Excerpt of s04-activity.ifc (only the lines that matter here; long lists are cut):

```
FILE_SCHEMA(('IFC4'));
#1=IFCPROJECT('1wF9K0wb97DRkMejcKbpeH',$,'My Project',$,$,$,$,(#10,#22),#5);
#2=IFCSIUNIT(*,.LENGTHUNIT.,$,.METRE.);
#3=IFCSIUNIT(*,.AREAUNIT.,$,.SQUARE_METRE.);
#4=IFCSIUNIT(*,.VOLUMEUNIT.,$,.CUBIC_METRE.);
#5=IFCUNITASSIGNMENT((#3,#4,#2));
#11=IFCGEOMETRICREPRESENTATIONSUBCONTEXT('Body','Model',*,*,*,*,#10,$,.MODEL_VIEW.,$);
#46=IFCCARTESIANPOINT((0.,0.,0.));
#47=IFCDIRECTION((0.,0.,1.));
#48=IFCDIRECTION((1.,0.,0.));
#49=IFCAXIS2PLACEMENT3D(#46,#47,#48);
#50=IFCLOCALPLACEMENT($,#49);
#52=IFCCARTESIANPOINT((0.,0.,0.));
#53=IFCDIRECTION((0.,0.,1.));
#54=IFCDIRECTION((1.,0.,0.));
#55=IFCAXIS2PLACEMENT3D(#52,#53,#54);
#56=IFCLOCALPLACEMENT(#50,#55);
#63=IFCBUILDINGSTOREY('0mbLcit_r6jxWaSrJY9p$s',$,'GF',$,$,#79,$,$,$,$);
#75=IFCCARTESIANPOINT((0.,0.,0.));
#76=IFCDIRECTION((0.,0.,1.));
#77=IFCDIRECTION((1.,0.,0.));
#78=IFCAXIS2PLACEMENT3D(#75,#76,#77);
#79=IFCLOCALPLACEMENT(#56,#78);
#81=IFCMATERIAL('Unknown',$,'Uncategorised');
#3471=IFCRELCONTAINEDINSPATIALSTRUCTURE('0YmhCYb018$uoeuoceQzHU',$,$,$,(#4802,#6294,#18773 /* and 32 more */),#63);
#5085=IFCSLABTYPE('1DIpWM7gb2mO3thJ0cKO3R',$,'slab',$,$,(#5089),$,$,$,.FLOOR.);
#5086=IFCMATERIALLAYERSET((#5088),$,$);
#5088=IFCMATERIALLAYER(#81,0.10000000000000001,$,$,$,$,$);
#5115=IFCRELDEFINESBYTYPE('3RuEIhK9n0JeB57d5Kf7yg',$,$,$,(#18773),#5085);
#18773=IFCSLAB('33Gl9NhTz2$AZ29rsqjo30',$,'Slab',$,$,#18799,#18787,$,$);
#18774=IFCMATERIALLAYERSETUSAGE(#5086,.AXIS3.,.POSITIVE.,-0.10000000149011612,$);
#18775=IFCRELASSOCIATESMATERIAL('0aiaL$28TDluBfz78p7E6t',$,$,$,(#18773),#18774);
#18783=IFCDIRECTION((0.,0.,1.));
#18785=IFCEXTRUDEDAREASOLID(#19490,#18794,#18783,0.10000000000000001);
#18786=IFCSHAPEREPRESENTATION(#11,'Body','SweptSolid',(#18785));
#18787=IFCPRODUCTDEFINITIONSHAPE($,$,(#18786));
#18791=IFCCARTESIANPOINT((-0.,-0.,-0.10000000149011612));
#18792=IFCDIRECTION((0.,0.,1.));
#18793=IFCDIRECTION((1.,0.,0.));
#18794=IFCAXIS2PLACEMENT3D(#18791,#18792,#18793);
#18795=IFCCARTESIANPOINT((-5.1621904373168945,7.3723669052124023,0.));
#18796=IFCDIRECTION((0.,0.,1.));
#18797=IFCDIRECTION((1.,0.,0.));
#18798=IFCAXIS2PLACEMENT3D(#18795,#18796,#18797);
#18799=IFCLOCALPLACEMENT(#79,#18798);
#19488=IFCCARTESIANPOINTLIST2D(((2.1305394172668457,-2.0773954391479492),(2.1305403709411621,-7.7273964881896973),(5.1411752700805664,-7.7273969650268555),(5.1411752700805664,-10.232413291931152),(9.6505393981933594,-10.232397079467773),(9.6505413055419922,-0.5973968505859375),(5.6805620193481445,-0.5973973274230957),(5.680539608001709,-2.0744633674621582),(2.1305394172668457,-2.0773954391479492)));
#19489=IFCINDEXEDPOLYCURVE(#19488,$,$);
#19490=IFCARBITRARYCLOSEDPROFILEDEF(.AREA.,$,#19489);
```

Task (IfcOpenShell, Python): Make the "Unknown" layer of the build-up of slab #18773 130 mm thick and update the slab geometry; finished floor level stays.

```python
import ifcopenshell
import ifcopenshell.util.element
import ifcopenshell.util.representation
import ifcopenshell.util.unit

model = ifcopenshell.open("s04-activity.ifc")
unit_scale = ifcopenshell.util.unit.calculate_unit_scale(model)

layer_set = model.by_id(5086)
layer = next(l for l in layer_set.MaterialLayers if l.Material and l.Material.Name == "Unknown")
change = 0.13 / unit_scale - layer.LayerThickness
layer.LayerThickness += change

# Geometry does not follow the layer set by itself.
slabs = [e for e in ifcopenshell.util.element.get_elements_by_material(model, layer_set) if e.is_a("IfcSlab")]
for slab in sorted(slabs, key=lambda e: e.id()):
    body = ifcopenshell.util.representation.get_representation(slab, "Model", "Body")
    solid = body.Items[0]
    old_depth = solid.Depth
    solid.Depth += change
    # Extruded upwards: lower the start of the extrusion so the top stays.
    x, y, z = solid.Position.Location.Coordinates
    solid.Position.Location = model.createIfcCartesianPoint((x, y, z - change))
    print(slab.id(), f"{old_depth:g} -> {solid.Depth:g}")

# The layers are counted up from the underside, which has moved.
for usage in {ifcopenshell.util.element.get_material(slab) for slab in slabs}:
    usage.OffsetFromReferenceLine -= change

model.write("s04-activity_edited.ifc")
```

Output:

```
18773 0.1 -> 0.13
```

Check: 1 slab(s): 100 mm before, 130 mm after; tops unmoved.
